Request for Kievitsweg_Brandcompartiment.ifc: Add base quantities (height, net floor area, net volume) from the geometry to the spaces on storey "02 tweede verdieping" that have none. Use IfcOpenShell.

First a look at what the model holds.

```python
import ifcopenshell
import ifcopenshell.util.element
import ifcopenshell.util.unit

model = ifcopenshell.open("Kievitsweg_Brandcompartiment.ifc")
print(model.schema)
for unit_type in ("LENGTHUNIT", "AREAUNIT", "VOLUMEUNIT"):
    print(unit_type, ifcopenshell.util.unit.calculate_unit_scale(model, unit_type))
storey = next(s for s in model.by_type("IfcBuildingStorey") if s.Name == "02 tweede verdieping")
spaces = [e for e in ifcopenshell.util.element.get_decomposition(storey) if e.is_a("IfcSpace")]
for e in sorted(spaces, key=lambda e: e.id()):
    print(e.id(), e.is_a(), e.Name, list(ifcopenshell.util.element.get_psets(e, qtos_only=True)), sep=" | ")
```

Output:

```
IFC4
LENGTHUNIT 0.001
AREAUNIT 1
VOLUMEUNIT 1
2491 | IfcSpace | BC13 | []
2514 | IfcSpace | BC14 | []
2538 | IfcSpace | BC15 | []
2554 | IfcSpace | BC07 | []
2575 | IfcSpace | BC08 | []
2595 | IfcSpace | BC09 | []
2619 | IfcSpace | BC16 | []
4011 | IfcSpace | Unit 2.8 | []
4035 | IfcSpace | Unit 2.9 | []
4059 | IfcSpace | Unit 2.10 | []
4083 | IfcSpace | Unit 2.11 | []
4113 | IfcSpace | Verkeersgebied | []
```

```python
import ifcopenshell
import ifcopenshell.api.pset
import ifcopenshell.geom
import ifcopenshell.util.element
import ifcopenshell.util.shape
import ifcopenshell.util.unit

model = ifcopenshell.open("Kievitsweg_Brandcompartiment.ifc")
unit_scale = ifcopenshell.util.unit.calculate_unit_scale(model)
area_scale = ifcopenshell.util.unit.calculate_unit_scale(model, "AREAUNIT")
volume_scale = ifcopenshell.util.unit.calculate_unit_scale(model, "VOLUMEUNIT")
settings = ifcopenshell.geom.settings()

storey = next(s for s in model.by_type("IfcBuildingStorey") if s.Name == "02 tweede verdieping")
spaces = [e for e in ifcopenshell.util.element.get_decomposition(storey) if e.is_a("IfcSpace")]

for e in sorted(spaces, key=lambda e: e.id()):
    if ifcopenshell.util.element.get_psets(e, qtos_only=True, should_inherit=False):
        continue
    # Geometry comes back in metres, in the element's own axes.
    shape = ifcopenshell.geom.create_shape(settings, e)
    values = {
        "Height": ifcopenshell.util.shape.get_z(shape.geometry) / unit_scale,
        "NetFloorArea": ifcopenshell.util.shape.get_footprint_area(shape.geometry) / area_scale,
        "NetVolume": ifcopenshell.util.shape.get_volume(shape.geometry) / volume_scale,
    }
    qto = ifcopenshell.api.pset.add_qto(model, product=e, name="Qto_SpaceBaseQuantities")
    ifcopenshell.api.pset.edit_qto(model, qto=qto, properties=values)
    print(e.id(), {k: round(v, 3) for k, v in values.items()})

model.write("Kievitsweg_Brandcompartiment_edited.ifc")
```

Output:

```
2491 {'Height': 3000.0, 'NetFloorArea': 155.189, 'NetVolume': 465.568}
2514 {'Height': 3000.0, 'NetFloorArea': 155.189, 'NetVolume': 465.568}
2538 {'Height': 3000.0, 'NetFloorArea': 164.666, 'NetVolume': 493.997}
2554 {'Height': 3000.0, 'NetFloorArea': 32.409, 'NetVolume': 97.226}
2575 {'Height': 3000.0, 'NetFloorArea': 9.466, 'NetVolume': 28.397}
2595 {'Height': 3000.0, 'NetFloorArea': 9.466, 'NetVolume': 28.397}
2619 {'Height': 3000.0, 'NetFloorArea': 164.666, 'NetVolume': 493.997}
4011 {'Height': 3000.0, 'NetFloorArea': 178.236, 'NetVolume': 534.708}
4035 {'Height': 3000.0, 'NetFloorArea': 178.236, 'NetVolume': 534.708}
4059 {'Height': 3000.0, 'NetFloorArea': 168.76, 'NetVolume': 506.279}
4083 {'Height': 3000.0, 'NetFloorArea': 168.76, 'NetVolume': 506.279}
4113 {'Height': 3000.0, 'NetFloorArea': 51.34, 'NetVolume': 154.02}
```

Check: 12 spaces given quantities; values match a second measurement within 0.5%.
